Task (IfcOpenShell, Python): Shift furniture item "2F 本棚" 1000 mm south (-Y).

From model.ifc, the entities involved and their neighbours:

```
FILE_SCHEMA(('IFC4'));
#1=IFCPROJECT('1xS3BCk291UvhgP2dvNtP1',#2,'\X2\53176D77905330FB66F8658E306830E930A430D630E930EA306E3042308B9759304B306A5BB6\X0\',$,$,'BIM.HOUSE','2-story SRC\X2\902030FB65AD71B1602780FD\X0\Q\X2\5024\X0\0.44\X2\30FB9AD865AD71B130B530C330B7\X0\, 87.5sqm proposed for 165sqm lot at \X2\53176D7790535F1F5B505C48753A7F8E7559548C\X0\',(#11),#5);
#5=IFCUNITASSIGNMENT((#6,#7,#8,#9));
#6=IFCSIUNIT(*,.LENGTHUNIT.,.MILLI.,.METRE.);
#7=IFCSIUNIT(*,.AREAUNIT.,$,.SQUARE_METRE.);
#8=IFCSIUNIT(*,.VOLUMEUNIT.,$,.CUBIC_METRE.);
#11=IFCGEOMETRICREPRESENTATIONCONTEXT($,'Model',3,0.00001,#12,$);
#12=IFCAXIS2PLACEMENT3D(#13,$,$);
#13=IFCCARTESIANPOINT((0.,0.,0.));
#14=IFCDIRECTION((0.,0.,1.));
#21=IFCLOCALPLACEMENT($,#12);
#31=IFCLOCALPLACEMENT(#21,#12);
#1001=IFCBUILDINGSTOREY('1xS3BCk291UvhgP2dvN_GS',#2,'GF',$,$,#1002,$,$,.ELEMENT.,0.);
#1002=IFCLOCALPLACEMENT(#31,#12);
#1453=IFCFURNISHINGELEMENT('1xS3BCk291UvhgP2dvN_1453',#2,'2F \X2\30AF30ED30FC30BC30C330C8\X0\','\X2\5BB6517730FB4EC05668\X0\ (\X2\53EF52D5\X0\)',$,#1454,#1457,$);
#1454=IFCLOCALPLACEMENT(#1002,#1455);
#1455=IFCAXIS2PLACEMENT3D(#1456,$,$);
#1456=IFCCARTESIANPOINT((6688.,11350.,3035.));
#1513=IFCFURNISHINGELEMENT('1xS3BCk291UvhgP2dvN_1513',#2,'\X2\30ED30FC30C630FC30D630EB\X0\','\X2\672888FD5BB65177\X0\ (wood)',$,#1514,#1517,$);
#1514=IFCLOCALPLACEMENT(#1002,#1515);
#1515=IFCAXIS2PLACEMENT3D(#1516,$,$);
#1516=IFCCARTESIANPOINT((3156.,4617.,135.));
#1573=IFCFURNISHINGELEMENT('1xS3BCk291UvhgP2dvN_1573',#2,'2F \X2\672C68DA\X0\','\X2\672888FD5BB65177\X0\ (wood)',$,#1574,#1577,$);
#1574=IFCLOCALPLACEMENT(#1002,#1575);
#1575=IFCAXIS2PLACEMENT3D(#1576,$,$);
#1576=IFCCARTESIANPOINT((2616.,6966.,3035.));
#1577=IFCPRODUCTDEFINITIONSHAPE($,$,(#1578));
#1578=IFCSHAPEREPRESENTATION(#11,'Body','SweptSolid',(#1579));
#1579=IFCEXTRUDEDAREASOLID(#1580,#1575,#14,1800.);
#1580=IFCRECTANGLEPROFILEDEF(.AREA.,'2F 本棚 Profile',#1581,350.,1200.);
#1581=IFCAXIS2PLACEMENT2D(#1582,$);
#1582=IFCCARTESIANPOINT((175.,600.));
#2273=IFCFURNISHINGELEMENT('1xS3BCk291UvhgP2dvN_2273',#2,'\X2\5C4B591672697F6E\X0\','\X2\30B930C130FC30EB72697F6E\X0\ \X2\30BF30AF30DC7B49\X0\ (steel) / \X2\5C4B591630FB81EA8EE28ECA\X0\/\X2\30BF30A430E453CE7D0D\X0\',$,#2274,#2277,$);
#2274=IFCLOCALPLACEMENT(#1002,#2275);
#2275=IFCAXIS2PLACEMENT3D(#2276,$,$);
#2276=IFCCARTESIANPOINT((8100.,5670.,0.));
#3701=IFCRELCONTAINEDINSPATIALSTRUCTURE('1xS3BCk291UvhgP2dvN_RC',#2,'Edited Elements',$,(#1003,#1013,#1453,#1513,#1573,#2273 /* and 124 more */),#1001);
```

```python
import ifcopenshell
import ifcopenshell.api.geometry
import ifcopenshell.util.placement

model = ifcopenshell.open("model.ifc")

item = model.by_guid("1xS3BCk291UvhgP2dvN_1573")
matrix = ifcopenshell.util.placement.get_local_placement(item.ObjectPlacement)
matrix[1, 3] -= 1000.0
ifcopenshell.api.geometry.edit_object_placement(model, product=item, matrix=matrix, is_si=False)

print(ifcopenshell.util.placement.get_local_placement(item.ObjectPlacement).round(3) + 0.0)

model.write("model-out.ifc")
```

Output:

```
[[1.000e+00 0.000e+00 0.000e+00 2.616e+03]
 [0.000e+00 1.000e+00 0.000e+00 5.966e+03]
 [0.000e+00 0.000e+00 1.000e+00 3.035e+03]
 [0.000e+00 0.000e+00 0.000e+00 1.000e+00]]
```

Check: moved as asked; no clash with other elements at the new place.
